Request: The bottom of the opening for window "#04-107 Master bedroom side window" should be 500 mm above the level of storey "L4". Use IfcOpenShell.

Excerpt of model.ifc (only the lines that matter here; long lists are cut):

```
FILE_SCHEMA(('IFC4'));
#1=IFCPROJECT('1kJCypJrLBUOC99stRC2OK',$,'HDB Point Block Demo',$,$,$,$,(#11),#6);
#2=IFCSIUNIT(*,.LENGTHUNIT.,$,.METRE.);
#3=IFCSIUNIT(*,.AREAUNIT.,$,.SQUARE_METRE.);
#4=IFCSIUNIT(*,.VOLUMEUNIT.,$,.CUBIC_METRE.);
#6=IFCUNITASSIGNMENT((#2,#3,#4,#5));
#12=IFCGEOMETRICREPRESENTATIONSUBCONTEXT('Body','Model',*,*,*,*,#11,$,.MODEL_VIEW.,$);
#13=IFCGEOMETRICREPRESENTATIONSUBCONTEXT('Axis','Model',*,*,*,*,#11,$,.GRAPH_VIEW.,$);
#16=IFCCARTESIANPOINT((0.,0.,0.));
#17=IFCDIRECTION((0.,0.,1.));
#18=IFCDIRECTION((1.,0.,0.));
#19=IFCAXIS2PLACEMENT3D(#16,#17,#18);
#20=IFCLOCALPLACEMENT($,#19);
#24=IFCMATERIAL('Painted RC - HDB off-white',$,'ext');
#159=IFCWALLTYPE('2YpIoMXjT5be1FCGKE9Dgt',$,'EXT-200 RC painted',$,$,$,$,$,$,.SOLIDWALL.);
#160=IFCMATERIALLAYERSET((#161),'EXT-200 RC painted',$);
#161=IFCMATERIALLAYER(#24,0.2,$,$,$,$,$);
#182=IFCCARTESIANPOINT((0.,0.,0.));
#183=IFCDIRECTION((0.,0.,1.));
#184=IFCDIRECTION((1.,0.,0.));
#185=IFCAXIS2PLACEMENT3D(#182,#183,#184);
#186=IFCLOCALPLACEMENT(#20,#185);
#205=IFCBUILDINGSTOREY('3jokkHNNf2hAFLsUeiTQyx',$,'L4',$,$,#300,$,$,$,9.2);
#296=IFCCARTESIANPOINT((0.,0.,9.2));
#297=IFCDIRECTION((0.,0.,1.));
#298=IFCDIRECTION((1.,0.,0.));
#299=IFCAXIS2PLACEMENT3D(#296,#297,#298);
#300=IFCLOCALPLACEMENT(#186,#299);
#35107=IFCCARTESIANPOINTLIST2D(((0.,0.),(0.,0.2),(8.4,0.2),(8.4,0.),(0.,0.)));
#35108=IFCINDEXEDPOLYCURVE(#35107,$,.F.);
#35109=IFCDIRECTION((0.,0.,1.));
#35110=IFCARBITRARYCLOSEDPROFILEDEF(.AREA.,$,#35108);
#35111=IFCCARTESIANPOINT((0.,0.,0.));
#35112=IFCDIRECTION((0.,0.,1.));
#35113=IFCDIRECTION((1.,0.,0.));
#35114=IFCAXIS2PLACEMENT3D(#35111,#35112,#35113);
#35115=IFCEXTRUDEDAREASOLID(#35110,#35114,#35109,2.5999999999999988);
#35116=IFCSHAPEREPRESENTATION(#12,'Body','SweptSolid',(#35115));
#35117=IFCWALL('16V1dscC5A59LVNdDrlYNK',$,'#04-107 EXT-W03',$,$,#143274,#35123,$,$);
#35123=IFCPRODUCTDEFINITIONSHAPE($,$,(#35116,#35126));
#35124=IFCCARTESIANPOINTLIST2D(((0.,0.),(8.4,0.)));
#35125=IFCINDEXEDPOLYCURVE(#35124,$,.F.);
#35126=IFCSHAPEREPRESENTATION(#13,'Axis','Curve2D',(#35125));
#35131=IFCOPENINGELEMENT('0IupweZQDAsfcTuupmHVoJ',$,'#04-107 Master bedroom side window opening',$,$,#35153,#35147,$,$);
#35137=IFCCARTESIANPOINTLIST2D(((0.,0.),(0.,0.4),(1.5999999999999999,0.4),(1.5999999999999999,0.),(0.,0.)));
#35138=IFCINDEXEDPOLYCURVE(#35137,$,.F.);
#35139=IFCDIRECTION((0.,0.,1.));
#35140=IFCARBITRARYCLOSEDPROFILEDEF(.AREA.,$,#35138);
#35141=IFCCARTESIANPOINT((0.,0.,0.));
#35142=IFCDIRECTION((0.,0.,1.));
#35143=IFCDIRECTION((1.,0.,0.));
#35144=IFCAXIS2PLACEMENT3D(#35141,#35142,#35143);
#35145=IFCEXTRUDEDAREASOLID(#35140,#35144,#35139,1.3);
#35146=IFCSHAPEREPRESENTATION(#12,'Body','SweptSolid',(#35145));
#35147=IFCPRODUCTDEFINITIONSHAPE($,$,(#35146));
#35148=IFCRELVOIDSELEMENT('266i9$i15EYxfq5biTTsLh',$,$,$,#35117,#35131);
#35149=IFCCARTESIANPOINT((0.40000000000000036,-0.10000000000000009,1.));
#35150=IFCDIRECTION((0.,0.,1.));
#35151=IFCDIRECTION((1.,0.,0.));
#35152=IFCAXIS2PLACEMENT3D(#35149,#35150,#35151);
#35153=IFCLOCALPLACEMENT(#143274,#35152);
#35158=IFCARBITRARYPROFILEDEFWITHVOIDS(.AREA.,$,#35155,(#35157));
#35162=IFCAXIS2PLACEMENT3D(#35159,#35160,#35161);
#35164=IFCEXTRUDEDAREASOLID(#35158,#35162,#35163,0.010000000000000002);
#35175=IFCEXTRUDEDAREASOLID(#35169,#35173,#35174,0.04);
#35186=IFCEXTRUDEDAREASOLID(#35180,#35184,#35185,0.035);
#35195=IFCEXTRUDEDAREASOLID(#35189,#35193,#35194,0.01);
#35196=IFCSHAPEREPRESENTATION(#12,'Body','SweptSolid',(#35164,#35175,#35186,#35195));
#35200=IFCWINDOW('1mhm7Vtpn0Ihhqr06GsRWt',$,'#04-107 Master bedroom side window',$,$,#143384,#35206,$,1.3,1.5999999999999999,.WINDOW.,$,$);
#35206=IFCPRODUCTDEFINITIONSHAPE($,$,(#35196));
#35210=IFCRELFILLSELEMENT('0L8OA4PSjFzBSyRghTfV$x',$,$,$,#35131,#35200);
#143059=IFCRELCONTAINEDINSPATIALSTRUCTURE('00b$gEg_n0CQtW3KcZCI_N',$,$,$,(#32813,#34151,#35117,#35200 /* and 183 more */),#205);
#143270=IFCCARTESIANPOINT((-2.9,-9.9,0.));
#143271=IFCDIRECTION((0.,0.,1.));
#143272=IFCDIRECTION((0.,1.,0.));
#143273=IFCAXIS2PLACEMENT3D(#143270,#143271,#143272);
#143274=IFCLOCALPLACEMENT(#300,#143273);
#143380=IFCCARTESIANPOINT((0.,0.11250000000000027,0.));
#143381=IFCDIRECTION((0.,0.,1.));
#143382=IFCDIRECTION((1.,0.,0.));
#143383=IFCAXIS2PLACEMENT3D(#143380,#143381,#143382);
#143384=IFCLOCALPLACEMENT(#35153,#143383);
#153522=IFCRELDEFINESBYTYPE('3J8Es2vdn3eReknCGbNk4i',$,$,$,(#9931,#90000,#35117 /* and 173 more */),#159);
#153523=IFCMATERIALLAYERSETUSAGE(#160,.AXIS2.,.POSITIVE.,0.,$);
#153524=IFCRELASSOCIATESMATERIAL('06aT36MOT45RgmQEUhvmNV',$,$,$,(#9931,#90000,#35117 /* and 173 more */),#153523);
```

```python
import numpy as np
import ifcopenshell
import ifcopenshell.api.geometry
import ifcopenshell.geom
import ifcopenshell.util.element
import ifcopenshell.util.placement
import ifcopenshell.util.shape
import ifcopenshell.util.unit

model = ifcopenshell.open("model.ifc")
unit_scale = ifcopenshell.util.unit.calculate_unit_scale(model)

window = model.by_id(35200)
opening = window.FillsVoids[0].RelatingOpeningElement
storey = ifcopenshell.util.element.get_container(window, ifc_class="IfcBuildingStorey")
level = ifcopenshell.util.placement.get_local_placement(storey.ObjectPlacement)[2, 3]

# The opening's origin need not be at the sill, so measure its lowest point.
shape = ifcopenshell.geom.create_shape(ifcopenshell.geom.settings(), opening)
bottom = ifcopenshell.util.shape.get_shape_bottom_elevation(shape, shape.geometry) / unit_scale
dz = level + 0.5 / unit_scale - bottom

shift = np.array([0.0, 0.0, dz])
# The window is placed relative to its opening, so it follows when the opening moves.
matrix = ifcopenshell.util.placement.get_local_placement(opening.ObjectPlacement)
matrix[:3, 3] += shift
ifcopenshell.api.geometry.edit_object_placement(
    model, product=opening, matrix=matrix, is_si=False, should_transform_children=True
)

print(f"moved by {dz * unit_scale:+.3f} m")

model.write("model-out.ifc")
```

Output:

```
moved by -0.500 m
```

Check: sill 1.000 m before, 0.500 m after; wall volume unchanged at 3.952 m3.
